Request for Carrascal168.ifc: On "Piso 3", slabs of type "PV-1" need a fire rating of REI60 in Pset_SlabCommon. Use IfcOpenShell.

First a look at what the model holds.

```python
import ifcopenshell
import ifcopenshell.util.element

model = ifcopenshell.open("Carrascal168.ifc")
print(model.schema)
storey = next(s for s in model.by_type("IfcBuildingStorey") if s.Name == "Piso 3")
slabs = [e for e in ifcopenshell.util.element.get_decomposition(storey) if e.is_a("IfcSlab")]
seen = {}
for e in slabs:
    element_type = ifcopenshell.util.element.get_type(e)
    key = (element_type.Name if element_type != e and element_type else None, ifcopenshell.util.element.get_pset(e, "Pset_SlabCommon", "FireRating"))
    seen[key] = seen.get(key, 0) + 1
for (name, value), count in sorted(seen.items(), key=str):
    print(count, "x", name, "|", value)
```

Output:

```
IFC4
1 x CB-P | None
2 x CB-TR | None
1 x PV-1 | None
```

```python
import ifcopenshell
import ifcopenshell.api.pset
import ifcopenshell.util.element

model = ifcopenshell.open("Carrascal168.ifc")

storey = next(s for s in model.by_type("IfcBuildingStorey") if s.Name == "Piso 3")
slabs = [e for e in ifcopenshell.util.element.get_decomposition(storey) if e.is_a("IfcSlab")]

count = 0
for e in slabs:
    element_type = ifcopenshell.util.element.get_type(e)
    if element_type in (None, e) or element_type.Name != "PV-1":
        continue
    # add_pset returns the element's existing set when there is one.
    pset = ifcopenshell.api.pset.add_pset(model, product=e, name="Pset_SlabCommon")
    ifcopenshell.api.pset.edit_pset(model, pset=pset, properties={"FireRating": "REI60"})
    count += 1

print(count, "slabs updated")

model.write("Carrascal168-out.ifc")
```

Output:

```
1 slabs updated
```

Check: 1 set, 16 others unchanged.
